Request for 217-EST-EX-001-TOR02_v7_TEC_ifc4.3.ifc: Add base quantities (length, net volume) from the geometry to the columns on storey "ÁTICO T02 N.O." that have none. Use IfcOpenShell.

First a look at what the model holds.

```python
import ifcopenshell
import ifcopenshell.util.element
import ifcopenshell.util.unit

model = ifcopenshell.open("217-EST-EX-001-TOR02_v7_TEC_ifc4.3.ifc")
print(model.schema)
for unit_type in ("LENGTHUNIT", "AREAUNIT", "VOLUMEUNIT"):
    print(unit_type, ifcopenshell.util.unit.calculate_unit_scale(model, unit_type))
storey = next(s for s in model.by_type("IfcBuildingStorey") if s.Name == "ÁTICO T02 N.O.")
columns = [e for e in ifcopenshell.util.element.get_decomposition(storey) if e.is_a("IfcColumn")]
for e in sorted(columns, key=lambda e: e.id()):
    print(e.id(), e.is_a(), e.Name, list(ifcopenshell.util.element.get_psets(e, qtos_only=True)), sep=" | ")
```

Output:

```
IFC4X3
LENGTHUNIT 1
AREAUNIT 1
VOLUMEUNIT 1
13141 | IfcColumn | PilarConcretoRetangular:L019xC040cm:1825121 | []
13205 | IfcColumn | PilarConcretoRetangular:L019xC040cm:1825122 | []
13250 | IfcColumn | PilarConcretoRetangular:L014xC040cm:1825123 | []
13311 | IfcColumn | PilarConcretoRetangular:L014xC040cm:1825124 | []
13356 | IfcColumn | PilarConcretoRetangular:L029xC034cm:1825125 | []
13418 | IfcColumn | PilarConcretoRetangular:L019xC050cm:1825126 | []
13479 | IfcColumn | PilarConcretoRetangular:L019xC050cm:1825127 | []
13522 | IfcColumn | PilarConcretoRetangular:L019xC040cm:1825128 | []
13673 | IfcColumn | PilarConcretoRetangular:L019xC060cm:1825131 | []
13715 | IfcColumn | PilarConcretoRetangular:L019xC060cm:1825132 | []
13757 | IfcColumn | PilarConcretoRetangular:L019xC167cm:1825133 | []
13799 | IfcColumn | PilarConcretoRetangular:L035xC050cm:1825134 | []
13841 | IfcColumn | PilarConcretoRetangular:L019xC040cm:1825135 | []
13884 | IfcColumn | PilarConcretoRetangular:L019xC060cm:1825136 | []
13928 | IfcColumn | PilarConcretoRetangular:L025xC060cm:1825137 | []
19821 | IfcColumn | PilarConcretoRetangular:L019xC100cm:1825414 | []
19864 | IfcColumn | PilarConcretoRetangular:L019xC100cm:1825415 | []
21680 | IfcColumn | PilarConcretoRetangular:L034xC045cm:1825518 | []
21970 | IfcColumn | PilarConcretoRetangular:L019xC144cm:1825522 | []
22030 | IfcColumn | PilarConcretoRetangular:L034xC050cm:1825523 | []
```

```python
import ifcopenshell
import ifcopenshell.api.pset
import ifcopenshell.geom
import ifcopenshell.util.element
import ifcopenshell.util.shape
import ifcopenshell.util.unit

model = ifcopenshell.open("217-EST-EX-001-TOR02_v7_TEC_ifc4.3.ifc")
unit_scale = ifcopenshell.util.unit.calculate_unit_scale(model)
volume_scale = ifcopenshell.util.unit.calculate_unit_scale(model, "VOLUMEUNIT")
settings = ifcopenshell.geom.settings()

storey = next(s for s in model.by_type("IfcBuildingStorey") if s.Name == "ÁTICO T02 N.O.")
columns = [e for e in ifcopenshell.util.element.get_decomposition(storey) if e.is_a("IfcColumn")]

for e in sorted(columns, key=lambda e: e.id()):
    if ifcopenshell.util.element.get_psets(e, qtos_only=True, should_inherit=False):
        continue
    # Geometry comes back in metres, in the element's own axes.
    shape = ifcopenshell.geom.create_shape(settings, e)
    values = {
        "Length": ifcopenshell.util.shape.get_z(shape.geometry) / unit_scale,
        "NetVolume": ifcopenshell.util.shape.get_volume(shape.geometry) / volume_scale,
    }
    qto = ifcopenshell.api.pset.add_qto(model, product=e, name="Qto_ColumnBaseQuantities")
    ifcopenshell.api.pset.edit_qto(model, qto=qto, properties=values)
    print(e.id(), {k: round(v, 3) for k, v in values.items()})

model.write("217-EST-EX-001-TOR02_v7_TEC_ifc4.3_updated.ifc")
```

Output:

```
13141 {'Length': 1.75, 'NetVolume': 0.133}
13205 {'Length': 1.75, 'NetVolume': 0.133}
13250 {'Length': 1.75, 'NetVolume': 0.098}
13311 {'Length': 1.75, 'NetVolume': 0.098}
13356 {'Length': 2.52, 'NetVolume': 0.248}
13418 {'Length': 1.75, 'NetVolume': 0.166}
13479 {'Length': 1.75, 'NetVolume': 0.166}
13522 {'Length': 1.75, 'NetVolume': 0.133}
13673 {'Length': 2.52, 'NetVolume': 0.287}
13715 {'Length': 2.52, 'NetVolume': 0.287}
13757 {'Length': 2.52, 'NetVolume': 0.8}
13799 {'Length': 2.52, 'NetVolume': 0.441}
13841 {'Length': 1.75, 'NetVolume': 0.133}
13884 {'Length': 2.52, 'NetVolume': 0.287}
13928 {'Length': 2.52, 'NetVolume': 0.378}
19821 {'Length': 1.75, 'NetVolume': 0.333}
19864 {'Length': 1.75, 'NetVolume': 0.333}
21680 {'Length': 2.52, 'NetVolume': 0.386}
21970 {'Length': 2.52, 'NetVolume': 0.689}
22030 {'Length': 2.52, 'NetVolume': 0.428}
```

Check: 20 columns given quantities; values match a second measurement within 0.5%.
